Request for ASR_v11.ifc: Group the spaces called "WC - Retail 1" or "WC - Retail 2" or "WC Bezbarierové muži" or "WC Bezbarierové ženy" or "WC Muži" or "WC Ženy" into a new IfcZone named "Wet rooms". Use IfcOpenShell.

First a look at what the model holds.

```python
import ifcopenshell

model = ifcopenshell.open("ASR_v11.ifc")
print(model.schema)
seen = {}
for space in model.by_type("IfcSpace"):
    seen[space.LongName] = seen.get(space.LongName, 0) + 1
for name, count in sorted(seen.items(), key=str):
    print(count, "x", name)
print("zones:", [z.Name for z in model.by_type("IfcZone")][:20])
```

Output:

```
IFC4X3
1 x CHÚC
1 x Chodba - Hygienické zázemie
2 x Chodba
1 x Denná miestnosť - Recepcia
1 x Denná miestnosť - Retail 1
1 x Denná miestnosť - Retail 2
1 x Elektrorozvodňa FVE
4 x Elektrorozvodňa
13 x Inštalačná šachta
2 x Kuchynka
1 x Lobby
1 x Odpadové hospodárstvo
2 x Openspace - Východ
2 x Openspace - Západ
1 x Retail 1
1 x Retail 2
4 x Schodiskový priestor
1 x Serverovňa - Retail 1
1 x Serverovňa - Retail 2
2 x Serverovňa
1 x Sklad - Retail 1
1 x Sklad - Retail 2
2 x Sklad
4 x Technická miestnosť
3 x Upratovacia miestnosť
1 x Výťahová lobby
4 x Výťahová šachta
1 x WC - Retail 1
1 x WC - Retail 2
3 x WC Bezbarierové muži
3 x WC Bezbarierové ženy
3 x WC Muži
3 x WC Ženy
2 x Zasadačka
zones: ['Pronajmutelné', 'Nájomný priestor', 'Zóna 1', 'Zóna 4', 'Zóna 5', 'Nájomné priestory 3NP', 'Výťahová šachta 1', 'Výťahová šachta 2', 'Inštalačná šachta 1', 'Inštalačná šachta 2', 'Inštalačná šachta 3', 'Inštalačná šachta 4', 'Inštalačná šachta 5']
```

```python
import ifcopenshell
import ifcopenshell.api.group
import ifcopenshell.api.root

model = ifcopenshell.open("ASR_v11.ifc")

names = {"WC - Retail 1", "WC - Retail 2", "WC Bezbarierové muži", "WC Bezbarierové ženy", "WC Muži", "WC Ženy"}
spaces = [s for s in model.by_type("IfcSpace") if s.LongName in names]

zone = ifcopenshell.api.root.create_entity(model, ifc_class="IfcZone", name="Wet rooms")
ifcopenshell.api.group.assign_group(model, products=spaces, group=zone)
print(len(spaces), "spaces in", zone.Name)

model.write("ASR_v11_rev.ifc")
```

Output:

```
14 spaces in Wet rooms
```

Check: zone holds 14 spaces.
